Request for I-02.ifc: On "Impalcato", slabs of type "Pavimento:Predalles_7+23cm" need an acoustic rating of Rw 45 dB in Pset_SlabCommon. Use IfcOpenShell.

First a look at what the model holds.

```python
import ifcopenshell
import ifcopenshell.util.element

model = ifcopenshell.open("I-02.ifc")
print(model.schema)
storey = next(s for s in model.by_type("IfcBuildingStorey") if s.Name == "Impalcato")
slabs = [e for e in ifcopenshell.util.element.get_decomposition(storey) if e.is_a("IfcSlab")]
seen = {}
for e in slabs:
    element_type = ifcopenshell.util.element.get_type(e)
    key = (element_type.Name if element_type != e and element_type else None, ifcopenshell.util.element.get_pset(e, "Pset_SlabCommon", "AcousticRating"))
    seen[key] = seen.get(key, 0) + 1
for (name, value), count in sorted(seen.items(), key=str):
    print(count, "x", name, "|", value)
```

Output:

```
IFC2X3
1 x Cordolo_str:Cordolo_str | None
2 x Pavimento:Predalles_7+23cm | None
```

```python
import ifcopenshell
import ifcopenshell.api.pset
import ifcopenshell.util.element

model = ifcopenshell.open("I-02.ifc")

storey = next(s for s in model.by_type("IfcBuildingStorey") if s.Name == "Impalcato")
slabs = [e for e in ifcopenshell.util.element.get_decomposition(storey) if e.is_a("IfcSlab")]

count = 0
for e in slabs:
    element_type = ifcopenshell.util.element.get_type(e)
    if element_type in (None, e) or element_type.Name != "Pavimento:Predalles_7+23cm":
        continue
    # add_pset returns the element's existing set when there is one.
    pset = ifcopenshell.api.pset.add_pset(model, product=e, name="Pset_SlabCommon")
    ifcopenshell.api.pset.edit_pset(model, pset=pset, properties={"AcousticRating": "Rw 45 dB"})
    count += 1

print(count, "slabs updated")

model.write("I-02_v2.ifc")
```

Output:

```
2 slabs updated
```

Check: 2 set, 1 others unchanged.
